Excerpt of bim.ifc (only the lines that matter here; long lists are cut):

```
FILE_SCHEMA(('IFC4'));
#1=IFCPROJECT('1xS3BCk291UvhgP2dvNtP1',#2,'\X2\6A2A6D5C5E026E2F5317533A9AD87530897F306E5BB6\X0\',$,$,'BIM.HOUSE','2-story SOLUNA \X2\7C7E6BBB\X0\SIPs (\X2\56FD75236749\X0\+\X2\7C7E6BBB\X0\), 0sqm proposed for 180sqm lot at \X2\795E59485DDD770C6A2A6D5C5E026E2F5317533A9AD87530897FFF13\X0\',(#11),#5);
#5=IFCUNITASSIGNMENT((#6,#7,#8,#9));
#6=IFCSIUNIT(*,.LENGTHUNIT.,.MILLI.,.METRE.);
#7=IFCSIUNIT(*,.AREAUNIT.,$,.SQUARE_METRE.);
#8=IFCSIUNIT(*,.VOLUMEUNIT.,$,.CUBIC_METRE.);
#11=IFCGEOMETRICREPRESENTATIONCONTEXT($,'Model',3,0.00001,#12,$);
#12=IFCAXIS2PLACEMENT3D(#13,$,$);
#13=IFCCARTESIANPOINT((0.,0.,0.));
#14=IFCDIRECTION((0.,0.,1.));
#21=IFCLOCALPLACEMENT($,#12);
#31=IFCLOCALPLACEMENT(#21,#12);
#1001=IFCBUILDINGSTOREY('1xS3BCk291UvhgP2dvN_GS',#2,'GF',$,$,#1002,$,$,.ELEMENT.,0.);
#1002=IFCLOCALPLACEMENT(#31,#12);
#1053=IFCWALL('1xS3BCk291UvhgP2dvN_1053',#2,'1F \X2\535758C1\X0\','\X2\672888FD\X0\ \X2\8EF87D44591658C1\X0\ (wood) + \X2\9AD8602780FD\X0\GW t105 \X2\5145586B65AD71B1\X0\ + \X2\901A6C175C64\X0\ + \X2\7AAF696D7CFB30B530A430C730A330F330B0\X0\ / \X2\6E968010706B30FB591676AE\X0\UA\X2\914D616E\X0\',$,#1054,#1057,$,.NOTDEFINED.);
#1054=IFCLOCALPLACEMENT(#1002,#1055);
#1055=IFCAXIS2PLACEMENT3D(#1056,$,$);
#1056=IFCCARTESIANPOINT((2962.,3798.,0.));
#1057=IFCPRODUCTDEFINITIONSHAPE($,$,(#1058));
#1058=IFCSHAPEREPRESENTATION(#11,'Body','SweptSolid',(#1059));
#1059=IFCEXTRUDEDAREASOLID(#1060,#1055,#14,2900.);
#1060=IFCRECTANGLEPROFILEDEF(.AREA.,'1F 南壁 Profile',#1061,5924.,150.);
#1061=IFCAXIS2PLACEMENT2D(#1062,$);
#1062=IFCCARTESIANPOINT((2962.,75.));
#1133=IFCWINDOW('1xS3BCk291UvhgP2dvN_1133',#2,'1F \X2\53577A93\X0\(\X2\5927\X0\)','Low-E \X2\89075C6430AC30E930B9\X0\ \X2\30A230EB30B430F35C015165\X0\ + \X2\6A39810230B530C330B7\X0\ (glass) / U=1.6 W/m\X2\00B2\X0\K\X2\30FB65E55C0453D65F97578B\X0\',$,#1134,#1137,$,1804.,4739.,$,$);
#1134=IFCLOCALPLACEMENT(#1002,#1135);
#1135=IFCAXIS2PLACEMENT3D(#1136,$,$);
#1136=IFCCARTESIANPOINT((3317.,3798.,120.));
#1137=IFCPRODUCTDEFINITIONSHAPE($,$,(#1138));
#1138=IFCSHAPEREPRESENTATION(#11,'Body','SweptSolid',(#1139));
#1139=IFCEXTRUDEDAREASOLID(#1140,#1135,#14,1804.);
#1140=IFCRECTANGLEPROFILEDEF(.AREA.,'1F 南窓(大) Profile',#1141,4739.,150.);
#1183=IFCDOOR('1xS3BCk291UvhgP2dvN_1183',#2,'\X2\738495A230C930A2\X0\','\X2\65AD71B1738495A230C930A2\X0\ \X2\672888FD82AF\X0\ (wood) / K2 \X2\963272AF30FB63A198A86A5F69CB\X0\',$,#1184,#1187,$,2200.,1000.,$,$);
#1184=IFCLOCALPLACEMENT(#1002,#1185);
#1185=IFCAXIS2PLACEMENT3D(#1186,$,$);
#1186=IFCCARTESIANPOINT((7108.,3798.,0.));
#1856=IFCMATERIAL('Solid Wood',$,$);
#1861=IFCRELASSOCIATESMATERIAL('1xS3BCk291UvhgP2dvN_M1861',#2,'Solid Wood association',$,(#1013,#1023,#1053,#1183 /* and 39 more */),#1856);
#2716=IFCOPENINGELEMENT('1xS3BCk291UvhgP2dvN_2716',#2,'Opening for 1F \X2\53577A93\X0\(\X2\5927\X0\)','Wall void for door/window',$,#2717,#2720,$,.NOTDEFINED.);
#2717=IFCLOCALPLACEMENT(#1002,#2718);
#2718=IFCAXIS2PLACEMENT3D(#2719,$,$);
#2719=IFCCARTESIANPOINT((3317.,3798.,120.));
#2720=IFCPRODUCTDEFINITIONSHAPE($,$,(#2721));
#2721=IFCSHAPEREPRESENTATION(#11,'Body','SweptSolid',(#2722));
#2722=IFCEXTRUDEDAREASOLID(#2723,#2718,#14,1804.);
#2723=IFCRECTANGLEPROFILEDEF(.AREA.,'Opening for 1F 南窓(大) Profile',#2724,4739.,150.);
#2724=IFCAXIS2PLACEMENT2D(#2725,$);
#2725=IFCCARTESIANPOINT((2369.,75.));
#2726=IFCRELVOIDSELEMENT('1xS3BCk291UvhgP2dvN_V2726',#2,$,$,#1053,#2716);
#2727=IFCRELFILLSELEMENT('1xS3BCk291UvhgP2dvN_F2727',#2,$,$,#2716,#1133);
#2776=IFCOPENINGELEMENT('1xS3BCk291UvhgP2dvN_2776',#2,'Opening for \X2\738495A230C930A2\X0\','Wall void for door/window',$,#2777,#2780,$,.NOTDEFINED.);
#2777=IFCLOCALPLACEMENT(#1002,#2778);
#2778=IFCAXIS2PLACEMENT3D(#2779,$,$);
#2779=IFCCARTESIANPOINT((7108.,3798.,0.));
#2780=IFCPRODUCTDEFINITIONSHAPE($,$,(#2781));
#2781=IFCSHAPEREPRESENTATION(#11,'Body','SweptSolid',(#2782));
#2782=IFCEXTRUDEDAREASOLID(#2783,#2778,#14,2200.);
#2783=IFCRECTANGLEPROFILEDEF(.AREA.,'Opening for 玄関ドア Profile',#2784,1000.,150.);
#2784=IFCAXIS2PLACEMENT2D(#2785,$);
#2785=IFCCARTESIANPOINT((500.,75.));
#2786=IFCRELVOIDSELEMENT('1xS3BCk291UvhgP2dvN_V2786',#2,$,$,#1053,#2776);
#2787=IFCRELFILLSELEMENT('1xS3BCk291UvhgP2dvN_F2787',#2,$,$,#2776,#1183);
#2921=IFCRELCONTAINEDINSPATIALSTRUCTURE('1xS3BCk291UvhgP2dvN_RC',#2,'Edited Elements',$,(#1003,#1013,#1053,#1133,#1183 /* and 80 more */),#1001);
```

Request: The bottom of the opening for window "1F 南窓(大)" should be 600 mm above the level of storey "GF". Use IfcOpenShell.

```python
import numpy as np
import ifcopenshell
import ifcopenshell.api.geometry
import ifcopenshell.geom
import ifcopenshell.util.element
import ifcopenshell.util.placement
import ifcopenshell.util.shape
import ifcopenshell.util.unit

model = ifcopenshell.open("bim.ifc")
unit_scale = ifcopenshell.util.unit.calculate_unit_scale(model)

window = model.by_guid("1xS3BCk291UvhgP2dvN_1133")
opening = window.FillsVoids[0].RelatingOpeningElement
storey = ifcopenshell.util.element.get_container(window, ifc_class="IfcBuildingStorey")
level = ifcopenshell.util.placement.get_local_placement(storey.ObjectPlacement)[2, 3]

# The opening's origin need not be at the sill, so measure its lowest point.
shape = ifcopenshell.geom.create_shape(ifcopenshell.geom.settings(), opening)
bottom = ifcopenshell.util.shape.get_shape_bottom_elevation(shape, shape.geometry) / unit_scale
dz = level + 0.6 / unit_scale - bottom

shift = np.array([0.0, 0.0, dz])
# The window is not placed relative to its opening, so move both.
for product in (opening, window):
    matrix = ifcopenshell.util.placement.get_local_placement(product.ObjectPlacement)
    matrix[:3, 3] += shift
    ifcopenshell.api.geometry.edit_object_placement(model, product=product, matrix=matrix, is_si=False)

print(f"moved by {dz * unit_scale:+.3f} m")

model.write("bim_v2.ifc")
```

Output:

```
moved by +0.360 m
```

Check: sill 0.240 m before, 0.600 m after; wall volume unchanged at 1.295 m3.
